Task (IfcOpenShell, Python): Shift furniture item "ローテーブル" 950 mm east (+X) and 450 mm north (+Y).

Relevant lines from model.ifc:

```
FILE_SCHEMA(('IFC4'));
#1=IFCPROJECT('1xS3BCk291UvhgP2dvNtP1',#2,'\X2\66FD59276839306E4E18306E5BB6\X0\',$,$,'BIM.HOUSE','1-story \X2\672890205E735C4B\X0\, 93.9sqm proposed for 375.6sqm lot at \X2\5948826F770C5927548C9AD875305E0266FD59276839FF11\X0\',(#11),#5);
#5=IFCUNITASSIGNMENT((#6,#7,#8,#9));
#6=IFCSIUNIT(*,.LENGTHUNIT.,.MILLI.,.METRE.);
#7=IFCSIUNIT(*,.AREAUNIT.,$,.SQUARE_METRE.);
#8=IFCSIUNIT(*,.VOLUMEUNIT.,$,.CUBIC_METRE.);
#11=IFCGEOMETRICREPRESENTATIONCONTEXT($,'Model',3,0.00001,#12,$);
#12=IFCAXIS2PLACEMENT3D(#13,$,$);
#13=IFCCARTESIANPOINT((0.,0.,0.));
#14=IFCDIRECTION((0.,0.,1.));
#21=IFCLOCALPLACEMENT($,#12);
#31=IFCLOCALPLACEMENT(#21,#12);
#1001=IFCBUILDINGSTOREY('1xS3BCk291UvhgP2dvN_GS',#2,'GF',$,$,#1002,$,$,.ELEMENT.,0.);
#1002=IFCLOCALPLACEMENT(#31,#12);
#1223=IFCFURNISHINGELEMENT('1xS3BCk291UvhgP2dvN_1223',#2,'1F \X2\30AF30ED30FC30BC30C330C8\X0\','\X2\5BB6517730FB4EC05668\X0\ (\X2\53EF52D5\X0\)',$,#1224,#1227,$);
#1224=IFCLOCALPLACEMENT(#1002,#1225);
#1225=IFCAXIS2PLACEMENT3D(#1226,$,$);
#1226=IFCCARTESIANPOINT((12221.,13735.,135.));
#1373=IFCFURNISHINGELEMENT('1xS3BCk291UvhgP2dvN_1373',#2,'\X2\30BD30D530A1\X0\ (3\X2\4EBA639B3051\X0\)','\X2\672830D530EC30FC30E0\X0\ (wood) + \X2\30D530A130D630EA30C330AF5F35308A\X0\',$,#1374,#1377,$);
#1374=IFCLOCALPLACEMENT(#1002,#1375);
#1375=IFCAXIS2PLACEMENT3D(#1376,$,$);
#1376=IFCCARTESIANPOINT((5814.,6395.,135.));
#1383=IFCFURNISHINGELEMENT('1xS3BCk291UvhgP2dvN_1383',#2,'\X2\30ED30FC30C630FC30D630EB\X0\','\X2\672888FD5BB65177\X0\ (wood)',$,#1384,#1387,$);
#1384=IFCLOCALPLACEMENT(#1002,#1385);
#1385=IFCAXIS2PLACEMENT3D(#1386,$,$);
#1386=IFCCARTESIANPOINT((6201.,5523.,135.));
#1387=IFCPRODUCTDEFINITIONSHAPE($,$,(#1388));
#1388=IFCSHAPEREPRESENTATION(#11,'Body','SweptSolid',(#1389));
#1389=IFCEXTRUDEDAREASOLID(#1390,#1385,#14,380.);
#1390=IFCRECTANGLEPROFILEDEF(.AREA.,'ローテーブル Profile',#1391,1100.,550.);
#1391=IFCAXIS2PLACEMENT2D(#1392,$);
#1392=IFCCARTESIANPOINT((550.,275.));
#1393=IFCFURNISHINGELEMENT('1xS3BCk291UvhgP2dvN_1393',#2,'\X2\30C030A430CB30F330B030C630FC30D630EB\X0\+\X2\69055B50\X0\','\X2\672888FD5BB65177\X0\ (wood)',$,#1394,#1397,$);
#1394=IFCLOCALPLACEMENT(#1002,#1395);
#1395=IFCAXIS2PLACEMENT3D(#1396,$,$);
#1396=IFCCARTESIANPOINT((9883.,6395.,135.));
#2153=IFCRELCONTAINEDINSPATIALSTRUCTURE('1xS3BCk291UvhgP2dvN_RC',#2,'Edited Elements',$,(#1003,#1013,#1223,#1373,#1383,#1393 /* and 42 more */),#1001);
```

```python
import ifcopenshell
import ifcopenshell.api.geometry
import ifcopenshell.util.placement

model = ifcopenshell.open("model.ifc")

item = model.by_id(1383)
matrix = ifcopenshell.util.placement.get_local_placement(item.ObjectPlacement)
matrix[0, 3] += 950.0
matrix[1, 3] += 450.0
ifcopenshell.api.geometry.edit_object_placement(model, product=item, matrix=matrix, is_si=False)

print(ifcopenshell.util.placement.get_local_placement(item.ObjectPlacement).round(3) + 0.0)

model.write("model_edited.ifc")
```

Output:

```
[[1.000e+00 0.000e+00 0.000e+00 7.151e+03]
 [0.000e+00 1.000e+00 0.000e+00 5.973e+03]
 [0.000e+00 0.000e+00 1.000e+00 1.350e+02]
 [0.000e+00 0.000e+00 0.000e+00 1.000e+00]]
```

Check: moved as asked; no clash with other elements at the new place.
